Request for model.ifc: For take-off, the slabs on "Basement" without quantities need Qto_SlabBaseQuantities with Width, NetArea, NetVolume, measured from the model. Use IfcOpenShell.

First a look at what the model holds.

```python
import ifcopenshell
import ifcopenshell.util.element
import ifcopenshell.util.unit

model = ifcopenshell.open("model.ifc")
print(model.schema)
for unit_type in ("LENGTHUNIT", "AREAUNIT", "VOLUMEUNIT"):
    print(unit_type, ifcopenshell.util.unit.calculate_unit_scale(model, unit_type))
storey = next(s for s in model.by_type("IfcBuildingStorey") if s.Name == "Basement")
slabs = [e for e in ifcopenshell.util.element.get_decomposition(storey) if e.is_a("IfcSlab")]
for e in sorted(slabs, key=lambda e: e.id()):
    print(e.id(), e.is_a(), e.Name, list(ifcopenshell.util.element.get_psets(e, qtos_only=True)), sep=" | ")
```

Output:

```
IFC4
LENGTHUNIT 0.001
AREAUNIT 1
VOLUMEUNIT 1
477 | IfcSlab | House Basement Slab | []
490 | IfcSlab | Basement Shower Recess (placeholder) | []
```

```python
import ifcopenshell
import ifcopenshell.api.pset
import ifcopenshell.geom
import ifcopenshell.util.element
import ifcopenshell.util.shape
import ifcopenshell.util.unit

model = ifcopenshell.open("model.ifc")
unit_scale = ifcopenshell.util.unit.calculate_unit_scale(model)
area_scale = ifcopenshell.util.unit.calculate_unit_scale(model, "AREAUNIT")
volume_scale = ifcopenshell.util.unit.calculate_unit_scale(model, "VOLUMEUNIT")
settings = ifcopenshell.geom.settings()

storey = next(s for s in model.by_type("IfcBuildingStorey") if s.Name == "Basement")
slabs = [e for e in ifcopenshell.util.element.get_decomposition(storey) if e.is_a("IfcSlab")]

for e in sorted(slabs, key=lambda e: e.id()):
    if ifcopenshell.util.element.get_psets(e, qtos_only=True, should_inherit=False):
        continue
    # Geometry comes back in metres, in the element's own axes.
    shape = ifcopenshell.geom.create_shape(settings, e)
    values = {
        "Width": ifcopenshell.util.shape.get_z(shape.geometry) / unit_scale,
        "NetArea": ifcopenshell.util.shape.get_footprint_area(shape.geometry) / area_scale,
        "NetVolume": ifcopenshell.util.shape.get_volume(shape.geometry) / volume_scale,
    }
    qto = ifcopenshell.api.pset.add_qto(model, product=e, name="Qto_SlabBaseQuantities")
    ifcopenshell.api.pset.edit_qto(model, qto=qto, properties=values)
    print(e.id(), {k: round(v, 3) for k, v in values.items()})

model.write("model-out.ifc")
```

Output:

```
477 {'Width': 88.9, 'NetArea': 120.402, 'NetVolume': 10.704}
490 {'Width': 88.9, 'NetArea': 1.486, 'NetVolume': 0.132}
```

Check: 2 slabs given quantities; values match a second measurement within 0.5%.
